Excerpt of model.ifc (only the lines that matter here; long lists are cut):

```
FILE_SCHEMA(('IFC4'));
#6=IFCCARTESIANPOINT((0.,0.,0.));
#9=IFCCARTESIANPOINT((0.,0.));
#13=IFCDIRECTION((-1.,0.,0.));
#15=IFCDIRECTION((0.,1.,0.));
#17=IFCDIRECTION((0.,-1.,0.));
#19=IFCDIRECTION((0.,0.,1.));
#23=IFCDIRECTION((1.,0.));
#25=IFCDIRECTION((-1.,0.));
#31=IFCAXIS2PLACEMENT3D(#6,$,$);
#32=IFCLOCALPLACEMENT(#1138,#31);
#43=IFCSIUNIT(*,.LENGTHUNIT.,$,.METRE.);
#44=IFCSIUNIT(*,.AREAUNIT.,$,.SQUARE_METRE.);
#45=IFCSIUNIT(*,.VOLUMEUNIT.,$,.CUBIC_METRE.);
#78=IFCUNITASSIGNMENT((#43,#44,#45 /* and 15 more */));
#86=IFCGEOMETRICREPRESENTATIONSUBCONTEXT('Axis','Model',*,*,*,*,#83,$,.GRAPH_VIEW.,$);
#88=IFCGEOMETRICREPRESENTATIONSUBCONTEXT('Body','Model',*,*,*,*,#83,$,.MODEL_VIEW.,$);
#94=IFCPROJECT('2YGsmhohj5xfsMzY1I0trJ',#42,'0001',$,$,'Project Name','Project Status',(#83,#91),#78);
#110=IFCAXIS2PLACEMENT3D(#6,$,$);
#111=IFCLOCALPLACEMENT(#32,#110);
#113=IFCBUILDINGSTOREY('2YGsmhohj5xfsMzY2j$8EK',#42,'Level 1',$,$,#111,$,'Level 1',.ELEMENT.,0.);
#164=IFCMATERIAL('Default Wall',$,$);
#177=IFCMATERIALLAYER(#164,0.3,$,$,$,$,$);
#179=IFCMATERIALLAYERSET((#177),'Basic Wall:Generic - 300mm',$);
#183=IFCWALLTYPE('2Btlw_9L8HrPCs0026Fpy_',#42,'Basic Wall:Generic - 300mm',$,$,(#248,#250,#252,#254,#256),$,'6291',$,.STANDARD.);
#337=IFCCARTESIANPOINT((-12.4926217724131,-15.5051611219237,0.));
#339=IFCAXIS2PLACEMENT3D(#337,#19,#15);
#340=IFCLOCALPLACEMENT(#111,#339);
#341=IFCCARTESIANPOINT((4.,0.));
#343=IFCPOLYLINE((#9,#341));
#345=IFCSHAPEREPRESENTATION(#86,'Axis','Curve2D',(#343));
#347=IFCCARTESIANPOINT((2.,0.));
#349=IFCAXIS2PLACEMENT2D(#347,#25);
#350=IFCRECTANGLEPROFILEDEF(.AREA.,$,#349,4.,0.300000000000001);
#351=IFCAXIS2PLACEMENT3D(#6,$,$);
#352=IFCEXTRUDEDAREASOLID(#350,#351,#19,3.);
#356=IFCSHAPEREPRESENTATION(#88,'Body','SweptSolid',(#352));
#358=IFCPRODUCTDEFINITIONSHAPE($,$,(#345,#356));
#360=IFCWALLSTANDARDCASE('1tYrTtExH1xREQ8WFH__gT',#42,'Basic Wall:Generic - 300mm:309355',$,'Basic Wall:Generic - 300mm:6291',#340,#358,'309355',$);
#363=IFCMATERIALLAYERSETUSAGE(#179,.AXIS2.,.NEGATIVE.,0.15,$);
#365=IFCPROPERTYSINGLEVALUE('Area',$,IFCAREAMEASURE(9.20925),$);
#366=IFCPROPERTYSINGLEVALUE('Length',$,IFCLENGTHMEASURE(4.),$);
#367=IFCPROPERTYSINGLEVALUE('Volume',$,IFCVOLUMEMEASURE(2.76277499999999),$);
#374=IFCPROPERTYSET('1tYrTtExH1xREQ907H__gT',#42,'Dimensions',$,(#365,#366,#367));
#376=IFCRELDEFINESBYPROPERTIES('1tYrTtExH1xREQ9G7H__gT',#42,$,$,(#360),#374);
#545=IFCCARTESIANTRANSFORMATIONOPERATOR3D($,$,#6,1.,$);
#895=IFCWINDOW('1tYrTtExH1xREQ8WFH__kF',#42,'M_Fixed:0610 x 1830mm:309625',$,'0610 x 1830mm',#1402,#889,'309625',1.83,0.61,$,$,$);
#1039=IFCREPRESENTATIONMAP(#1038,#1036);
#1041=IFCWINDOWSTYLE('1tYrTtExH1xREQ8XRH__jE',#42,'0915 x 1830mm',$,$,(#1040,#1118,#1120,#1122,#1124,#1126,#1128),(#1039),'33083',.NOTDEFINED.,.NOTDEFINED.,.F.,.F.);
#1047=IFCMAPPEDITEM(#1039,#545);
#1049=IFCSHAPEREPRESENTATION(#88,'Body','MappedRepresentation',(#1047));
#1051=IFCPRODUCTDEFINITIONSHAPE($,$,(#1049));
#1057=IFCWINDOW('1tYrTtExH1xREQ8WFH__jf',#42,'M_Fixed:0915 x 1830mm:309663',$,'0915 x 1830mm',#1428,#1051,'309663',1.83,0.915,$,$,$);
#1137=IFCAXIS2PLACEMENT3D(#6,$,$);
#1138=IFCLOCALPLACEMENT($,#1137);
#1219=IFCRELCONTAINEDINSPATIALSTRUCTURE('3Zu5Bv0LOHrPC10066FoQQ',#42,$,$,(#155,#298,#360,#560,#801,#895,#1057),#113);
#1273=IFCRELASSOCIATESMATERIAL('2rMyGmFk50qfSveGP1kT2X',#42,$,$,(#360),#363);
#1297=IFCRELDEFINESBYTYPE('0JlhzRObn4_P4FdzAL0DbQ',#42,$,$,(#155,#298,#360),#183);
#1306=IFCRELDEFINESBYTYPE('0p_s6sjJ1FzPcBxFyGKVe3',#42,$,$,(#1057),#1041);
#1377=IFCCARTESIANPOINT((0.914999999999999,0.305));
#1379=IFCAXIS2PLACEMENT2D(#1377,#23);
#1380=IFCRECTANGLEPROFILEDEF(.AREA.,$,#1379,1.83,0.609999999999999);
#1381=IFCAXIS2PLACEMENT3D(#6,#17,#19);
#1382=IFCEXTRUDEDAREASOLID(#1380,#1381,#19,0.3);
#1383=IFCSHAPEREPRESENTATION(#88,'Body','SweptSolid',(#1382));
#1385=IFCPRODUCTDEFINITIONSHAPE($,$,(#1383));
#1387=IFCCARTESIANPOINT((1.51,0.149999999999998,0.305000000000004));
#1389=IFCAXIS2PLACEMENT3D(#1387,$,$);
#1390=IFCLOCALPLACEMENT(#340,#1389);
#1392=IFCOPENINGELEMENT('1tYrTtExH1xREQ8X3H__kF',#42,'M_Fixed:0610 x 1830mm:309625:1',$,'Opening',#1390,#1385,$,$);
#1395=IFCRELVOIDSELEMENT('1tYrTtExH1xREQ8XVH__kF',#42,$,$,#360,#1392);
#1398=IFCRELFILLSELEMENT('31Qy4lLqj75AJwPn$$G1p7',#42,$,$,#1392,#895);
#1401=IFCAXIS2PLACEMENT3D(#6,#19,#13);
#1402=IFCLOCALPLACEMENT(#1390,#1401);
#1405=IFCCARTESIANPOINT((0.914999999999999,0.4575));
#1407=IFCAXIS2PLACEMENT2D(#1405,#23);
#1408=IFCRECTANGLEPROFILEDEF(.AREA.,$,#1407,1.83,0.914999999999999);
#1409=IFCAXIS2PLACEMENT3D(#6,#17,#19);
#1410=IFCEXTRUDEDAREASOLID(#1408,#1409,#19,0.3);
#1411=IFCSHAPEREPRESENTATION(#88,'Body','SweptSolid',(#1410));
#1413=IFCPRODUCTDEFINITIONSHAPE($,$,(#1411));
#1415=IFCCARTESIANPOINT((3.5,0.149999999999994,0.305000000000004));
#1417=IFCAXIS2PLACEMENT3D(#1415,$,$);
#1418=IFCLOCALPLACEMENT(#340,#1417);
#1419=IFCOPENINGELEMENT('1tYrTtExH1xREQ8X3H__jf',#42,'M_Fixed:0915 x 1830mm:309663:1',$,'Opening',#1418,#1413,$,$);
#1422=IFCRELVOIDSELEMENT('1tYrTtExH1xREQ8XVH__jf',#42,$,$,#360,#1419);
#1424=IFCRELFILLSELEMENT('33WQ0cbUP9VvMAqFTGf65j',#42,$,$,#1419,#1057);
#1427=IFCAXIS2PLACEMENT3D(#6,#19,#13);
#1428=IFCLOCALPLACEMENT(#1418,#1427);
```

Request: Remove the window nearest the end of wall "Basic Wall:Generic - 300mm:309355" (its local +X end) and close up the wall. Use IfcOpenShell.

```python
import ifcopenshell
import ifcopenshell.api.feature
import ifcopenshell.api.pset
import ifcopenshell.api.root
import ifcopenshell.geom
import ifcopenshell.util.element
import ifcopenshell.util.shape
import ifcopenshell.util.unit

model = ifcopenshell.open("model.ifc")
area_scale = ifcopenshell.util.unit.calculate_unit_scale(model, "AREAUNIT")
volume_scale = ifcopenshell.util.unit.calculate_unit_scale(model, "VOLUMEUNIT")
settings = ifcopenshell.geom.settings()


def volume(element):
    """Net volume in cubic metres, openings subtracted."""
    shape = ifcopenshell.geom.create_shape(settings, element)
    return ifcopenshell.util.shape.get_volume(shape.geometry)


window = model.by_guid("1tYrTtExH1xREQ8WFH__jf")
opening = window.FillsVoids[0].RelatingOpeningElement
wall = opening.VoidsElements[0].RelatingBuildingElement
before = volume(wall)

ifcopenshell.api.root.remove_product(model, product=window)
ifcopenshell.api.feature.remove_feature(model, feature=opening)

after = volume(wall)
thickness = 0.3  # wall thickness in metres

# Update the wall's stored quantities.
pset = model.by_id(ifcopenshell.util.element.get_pset(wall, "Dimensions", should_inherit=False)["id"])
ifcopenshell.api.pset.edit_pset(model, pset=pset, properties={
    "Area": model.create_entity("IfcAreaMeasure", after / thickness / area_scale),
    "Volume": model.create_entity("IfcVolumeMeasure", after / volume_scale),
})

print(f"wall volume {before:.3f} -> {after:.3f} m3")

model.write("model_updated.ifc")
```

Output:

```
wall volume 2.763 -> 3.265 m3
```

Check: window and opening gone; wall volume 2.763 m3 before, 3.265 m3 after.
